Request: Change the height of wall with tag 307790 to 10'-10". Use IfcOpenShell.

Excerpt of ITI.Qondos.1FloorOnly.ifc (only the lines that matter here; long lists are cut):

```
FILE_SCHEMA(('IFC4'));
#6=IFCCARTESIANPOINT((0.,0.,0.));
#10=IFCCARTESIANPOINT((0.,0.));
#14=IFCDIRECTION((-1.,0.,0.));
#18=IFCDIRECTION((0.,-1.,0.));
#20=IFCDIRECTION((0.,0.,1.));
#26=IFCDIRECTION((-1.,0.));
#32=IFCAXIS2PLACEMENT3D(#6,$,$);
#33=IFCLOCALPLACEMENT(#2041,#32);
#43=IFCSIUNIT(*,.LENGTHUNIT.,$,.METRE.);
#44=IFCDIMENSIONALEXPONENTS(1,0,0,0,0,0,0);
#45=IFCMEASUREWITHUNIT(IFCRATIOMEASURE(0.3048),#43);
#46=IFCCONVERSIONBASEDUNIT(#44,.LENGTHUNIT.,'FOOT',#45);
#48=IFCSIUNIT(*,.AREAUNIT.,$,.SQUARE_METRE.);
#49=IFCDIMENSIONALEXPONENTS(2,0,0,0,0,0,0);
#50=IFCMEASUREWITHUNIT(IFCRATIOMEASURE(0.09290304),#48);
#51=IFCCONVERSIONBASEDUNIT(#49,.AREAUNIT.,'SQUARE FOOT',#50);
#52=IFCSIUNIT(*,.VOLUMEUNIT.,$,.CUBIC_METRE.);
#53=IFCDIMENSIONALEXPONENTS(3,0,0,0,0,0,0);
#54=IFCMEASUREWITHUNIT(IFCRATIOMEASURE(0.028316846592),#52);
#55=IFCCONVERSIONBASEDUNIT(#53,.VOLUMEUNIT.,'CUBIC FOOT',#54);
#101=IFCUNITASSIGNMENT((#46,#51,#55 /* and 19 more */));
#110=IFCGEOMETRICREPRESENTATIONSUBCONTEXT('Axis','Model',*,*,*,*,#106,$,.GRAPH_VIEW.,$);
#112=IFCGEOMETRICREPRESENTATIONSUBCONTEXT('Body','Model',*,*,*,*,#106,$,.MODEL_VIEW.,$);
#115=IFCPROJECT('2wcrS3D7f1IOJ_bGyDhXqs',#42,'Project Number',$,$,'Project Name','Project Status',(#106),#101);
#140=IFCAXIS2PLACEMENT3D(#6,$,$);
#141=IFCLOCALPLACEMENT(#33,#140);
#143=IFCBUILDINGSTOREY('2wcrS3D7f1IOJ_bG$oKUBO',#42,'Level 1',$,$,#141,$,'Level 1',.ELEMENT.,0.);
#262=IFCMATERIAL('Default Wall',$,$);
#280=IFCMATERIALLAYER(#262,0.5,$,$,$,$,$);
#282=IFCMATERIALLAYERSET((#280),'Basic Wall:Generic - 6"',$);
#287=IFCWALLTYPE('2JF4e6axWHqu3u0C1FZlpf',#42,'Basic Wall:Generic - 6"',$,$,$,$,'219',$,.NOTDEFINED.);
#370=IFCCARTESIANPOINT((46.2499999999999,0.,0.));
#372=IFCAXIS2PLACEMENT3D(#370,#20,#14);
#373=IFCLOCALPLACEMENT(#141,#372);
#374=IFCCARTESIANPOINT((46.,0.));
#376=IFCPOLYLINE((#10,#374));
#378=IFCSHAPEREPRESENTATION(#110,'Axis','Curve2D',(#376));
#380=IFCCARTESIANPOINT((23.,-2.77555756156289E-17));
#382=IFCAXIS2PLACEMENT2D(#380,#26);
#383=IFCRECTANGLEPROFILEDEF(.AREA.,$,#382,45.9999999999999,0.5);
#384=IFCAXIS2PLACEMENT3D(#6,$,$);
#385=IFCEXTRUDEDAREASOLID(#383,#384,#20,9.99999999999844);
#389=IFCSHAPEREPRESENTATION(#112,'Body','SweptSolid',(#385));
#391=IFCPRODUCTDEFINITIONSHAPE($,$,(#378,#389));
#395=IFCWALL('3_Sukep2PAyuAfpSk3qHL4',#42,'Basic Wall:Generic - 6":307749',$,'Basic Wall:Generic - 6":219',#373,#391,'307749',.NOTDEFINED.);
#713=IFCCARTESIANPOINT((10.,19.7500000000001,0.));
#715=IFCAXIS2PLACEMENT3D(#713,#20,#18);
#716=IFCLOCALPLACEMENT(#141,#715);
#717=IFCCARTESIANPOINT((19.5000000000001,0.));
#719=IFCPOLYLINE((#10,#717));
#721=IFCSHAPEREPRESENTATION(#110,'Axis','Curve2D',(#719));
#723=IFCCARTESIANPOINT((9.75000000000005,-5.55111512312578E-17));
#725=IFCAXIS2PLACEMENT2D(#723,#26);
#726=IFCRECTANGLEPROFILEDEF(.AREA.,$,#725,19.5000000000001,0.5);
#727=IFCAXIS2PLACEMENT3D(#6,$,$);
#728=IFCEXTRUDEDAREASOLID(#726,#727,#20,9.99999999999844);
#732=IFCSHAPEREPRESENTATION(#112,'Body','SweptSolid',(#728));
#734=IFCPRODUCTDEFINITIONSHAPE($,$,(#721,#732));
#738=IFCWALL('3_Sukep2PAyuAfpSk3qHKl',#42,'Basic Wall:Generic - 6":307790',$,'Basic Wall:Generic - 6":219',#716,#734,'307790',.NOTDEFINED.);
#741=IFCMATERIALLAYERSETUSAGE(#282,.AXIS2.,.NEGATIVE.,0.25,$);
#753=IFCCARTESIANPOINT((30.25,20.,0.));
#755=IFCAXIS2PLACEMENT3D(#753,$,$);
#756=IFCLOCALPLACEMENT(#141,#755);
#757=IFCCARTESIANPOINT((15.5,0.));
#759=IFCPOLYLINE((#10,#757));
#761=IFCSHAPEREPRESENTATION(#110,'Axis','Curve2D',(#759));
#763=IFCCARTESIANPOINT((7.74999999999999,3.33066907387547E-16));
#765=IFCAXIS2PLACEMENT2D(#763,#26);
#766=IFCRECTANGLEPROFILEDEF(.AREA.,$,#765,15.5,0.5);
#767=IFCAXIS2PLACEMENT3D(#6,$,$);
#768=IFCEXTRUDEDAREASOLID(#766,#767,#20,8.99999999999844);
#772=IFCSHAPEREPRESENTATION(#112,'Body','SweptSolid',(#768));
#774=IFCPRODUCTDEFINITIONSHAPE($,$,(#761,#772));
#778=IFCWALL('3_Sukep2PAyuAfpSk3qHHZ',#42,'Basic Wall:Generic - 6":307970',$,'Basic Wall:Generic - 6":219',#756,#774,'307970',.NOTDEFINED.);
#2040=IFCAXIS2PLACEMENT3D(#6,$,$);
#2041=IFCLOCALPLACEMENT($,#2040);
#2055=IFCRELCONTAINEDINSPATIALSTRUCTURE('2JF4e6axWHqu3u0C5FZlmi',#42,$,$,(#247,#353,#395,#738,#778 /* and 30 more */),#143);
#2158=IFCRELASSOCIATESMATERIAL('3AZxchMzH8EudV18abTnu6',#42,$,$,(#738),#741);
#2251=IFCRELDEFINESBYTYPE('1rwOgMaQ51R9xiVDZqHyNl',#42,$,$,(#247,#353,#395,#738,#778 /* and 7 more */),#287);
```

```python
import ifcopenshell
import ifcopenshell.geom
import ifcopenshell.util.representation
import ifcopenshell.util.shape
import ifcopenshell.util.unit

model = ifcopenshell.open("ITI.Qondos.1FloorOnly.ifc")
unit_scale = ifcopenshell.util.unit.calculate_unit_scale(model)
settings = ifcopenshell.geom.settings()


def volume(element):
    """Net volume in cubic metres, openings subtracted."""
    shape = ifcopenshell.geom.create_shape(settings, element)
    return ifcopenshell.util.shape.get_volume(shape.geometry)


wall = model.by_guid("3_Sukep2PAyuAfpSk3qHKl")
before = volume(wall)

body = ifcopenshell.util.representation.get_representation(wall, "Model", "Body")
solid = body.Items[0]
old_height = solid.Depth
solid.Depth = 130 * 0.0254 / unit_scale
after = volume(wall)

print(f"height {old_height:g} -> {solid.Depth:g}, volume {before:.3f} -> {after:.3f} m3")

model.write("ITI.Qondos.1FloorOnly_rev.ifc")
```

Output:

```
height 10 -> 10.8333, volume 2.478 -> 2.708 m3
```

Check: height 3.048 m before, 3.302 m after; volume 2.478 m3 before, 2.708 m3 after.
